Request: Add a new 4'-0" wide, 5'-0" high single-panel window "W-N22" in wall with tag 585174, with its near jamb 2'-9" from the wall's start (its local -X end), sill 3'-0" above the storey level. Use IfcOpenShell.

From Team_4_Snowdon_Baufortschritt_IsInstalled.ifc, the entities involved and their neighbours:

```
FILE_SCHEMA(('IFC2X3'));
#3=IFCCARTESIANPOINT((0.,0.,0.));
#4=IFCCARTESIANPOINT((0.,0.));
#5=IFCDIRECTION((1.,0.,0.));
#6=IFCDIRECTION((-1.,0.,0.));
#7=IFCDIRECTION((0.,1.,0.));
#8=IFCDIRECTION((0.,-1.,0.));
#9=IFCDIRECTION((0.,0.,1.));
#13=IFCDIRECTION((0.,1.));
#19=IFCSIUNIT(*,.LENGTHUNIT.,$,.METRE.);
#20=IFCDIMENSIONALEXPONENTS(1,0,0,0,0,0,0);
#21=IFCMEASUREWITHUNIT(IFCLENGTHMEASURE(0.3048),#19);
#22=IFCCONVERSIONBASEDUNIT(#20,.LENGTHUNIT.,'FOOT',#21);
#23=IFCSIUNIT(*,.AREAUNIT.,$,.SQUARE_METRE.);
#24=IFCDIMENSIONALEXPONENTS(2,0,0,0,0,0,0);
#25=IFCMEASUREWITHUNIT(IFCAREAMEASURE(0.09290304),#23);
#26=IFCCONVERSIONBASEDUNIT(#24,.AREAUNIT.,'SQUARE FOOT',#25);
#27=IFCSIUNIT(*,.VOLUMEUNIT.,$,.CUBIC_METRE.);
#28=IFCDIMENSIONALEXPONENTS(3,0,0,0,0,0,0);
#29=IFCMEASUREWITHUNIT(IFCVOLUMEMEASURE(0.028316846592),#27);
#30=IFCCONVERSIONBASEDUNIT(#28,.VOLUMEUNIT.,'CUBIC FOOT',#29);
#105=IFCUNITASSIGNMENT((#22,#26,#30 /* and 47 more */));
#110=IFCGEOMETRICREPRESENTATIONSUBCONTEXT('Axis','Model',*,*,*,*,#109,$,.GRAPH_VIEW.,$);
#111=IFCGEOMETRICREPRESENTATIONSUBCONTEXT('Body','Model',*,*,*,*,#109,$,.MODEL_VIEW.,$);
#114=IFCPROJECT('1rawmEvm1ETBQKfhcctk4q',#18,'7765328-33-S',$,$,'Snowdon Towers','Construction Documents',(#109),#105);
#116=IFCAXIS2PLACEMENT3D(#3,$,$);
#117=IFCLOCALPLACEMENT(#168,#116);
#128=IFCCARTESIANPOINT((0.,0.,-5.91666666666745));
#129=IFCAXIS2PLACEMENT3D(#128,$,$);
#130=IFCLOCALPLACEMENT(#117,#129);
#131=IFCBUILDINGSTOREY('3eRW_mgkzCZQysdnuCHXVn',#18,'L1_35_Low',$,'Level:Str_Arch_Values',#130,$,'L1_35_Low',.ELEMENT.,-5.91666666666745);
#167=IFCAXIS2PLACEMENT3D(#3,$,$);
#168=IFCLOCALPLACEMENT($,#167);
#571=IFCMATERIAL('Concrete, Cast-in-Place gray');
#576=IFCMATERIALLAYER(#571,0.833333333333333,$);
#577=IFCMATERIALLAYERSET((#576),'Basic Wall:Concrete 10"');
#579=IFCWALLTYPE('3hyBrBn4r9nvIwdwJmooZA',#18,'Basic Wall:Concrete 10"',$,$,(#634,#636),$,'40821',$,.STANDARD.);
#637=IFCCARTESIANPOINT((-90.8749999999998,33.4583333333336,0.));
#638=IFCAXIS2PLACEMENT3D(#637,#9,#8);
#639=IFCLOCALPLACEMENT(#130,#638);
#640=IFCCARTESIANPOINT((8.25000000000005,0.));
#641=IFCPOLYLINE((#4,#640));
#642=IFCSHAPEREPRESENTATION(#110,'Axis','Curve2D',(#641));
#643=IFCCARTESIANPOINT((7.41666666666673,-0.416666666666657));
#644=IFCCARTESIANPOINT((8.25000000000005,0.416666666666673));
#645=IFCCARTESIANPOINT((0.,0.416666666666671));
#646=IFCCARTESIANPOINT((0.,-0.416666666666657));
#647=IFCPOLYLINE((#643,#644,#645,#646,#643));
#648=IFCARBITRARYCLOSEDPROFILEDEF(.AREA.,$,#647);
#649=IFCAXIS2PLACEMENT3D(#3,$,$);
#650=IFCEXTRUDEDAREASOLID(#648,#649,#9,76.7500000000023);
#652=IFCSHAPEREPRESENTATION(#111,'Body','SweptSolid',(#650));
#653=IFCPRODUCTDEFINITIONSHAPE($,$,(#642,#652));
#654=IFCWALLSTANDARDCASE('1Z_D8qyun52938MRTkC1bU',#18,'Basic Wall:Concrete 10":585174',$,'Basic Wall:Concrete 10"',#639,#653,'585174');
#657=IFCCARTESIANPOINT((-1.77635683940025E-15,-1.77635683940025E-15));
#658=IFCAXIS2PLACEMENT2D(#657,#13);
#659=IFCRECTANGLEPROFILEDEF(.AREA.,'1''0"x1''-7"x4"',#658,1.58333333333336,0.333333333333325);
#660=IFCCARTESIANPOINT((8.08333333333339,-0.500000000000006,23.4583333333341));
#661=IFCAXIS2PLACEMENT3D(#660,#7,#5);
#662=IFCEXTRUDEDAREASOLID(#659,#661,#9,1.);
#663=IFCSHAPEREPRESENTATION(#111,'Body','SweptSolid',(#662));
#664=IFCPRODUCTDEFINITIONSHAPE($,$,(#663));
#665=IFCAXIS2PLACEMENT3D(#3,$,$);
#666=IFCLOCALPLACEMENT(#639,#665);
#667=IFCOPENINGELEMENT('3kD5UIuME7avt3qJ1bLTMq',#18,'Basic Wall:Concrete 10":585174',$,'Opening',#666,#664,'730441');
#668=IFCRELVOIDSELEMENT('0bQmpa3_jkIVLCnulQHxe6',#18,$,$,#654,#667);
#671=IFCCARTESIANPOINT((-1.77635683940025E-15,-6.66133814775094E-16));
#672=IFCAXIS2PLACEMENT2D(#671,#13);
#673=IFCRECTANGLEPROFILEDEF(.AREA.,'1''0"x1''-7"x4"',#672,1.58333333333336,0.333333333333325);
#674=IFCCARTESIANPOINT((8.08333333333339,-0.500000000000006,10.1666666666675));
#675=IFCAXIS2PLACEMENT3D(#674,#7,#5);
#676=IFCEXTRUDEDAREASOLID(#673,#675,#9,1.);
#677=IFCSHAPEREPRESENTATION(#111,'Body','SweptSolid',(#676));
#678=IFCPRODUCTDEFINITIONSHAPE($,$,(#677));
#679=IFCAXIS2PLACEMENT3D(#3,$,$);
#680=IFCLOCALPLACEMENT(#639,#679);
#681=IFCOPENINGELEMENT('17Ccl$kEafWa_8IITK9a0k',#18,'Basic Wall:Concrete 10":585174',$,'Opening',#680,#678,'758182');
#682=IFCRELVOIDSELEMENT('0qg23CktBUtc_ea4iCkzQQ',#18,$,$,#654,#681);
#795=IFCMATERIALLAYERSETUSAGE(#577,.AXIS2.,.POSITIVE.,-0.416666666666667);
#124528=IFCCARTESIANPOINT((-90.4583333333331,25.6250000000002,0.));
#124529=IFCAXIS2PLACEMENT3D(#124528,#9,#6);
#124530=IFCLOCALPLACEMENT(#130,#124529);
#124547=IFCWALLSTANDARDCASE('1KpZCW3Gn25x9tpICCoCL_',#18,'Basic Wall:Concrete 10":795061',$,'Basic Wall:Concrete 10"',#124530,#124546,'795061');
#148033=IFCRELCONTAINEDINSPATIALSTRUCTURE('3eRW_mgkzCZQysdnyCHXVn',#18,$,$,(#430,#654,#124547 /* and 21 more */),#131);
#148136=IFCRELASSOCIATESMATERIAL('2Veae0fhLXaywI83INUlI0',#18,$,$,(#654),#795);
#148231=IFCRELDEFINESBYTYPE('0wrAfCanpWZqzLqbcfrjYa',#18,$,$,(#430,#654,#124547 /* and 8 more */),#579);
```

```python
import numpy as np
import ifcopenshell
import ifcopenshell.api.feature
import ifcopenshell.api.geometry
import ifcopenshell.api.root
import ifcopenshell.api.spatial
import ifcopenshell.api.type
import ifcopenshell.geom
import ifcopenshell.util.element
import ifcopenshell.util.placement
import ifcopenshell.util.representation
import ifcopenshell.util.shape
import ifcopenshell.util.unit

model = ifcopenshell.open("Team_4_Snowdon_Baufortschritt_IsInstalled.ifc")
unit_scale = ifcopenshell.util.unit.calculate_unit_scale(model)
settings = ifcopenshell.geom.settings()


def volume(element):
    """Net volume in cubic metres, openings subtracted."""
    shape = ifcopenshell.geom.create_shape(settings, element)
    return ifcopenshell.util.shape.get_volume(shape.geometry)


wall = model.by_guid("1Z_D8qyun52938MRTkC1bU")
storey = ifcopenshell.util.element.get_container(wall, ifc_class="IfcBuildingStorey")
context = ifcopenshell.util.representation.get_context(model, "Model", "Body", "MODEL_VIEW")
before = volume(wall)

width, height, from_end, sill = 1.2192, 1.524, 0.8382, 0.9144  # metres

# The wall runs along its own X axis, and the end named is its -X end.
wall_shape = ifcopenshell.geom.create_shape(settings, wall)
x, y, z = ifcopenshell.util.shape.get_vertices(wall_shape.geometry).T
start = x.min() + from_end
face, thickness = float(y.min()), float(y.max() - y.min())
wall_matrix = ifcopenshell.util.placement.get_local_placement(wall.ObjectPlacement)
level = ifcopenshell.util.placement.get_local_placement(storey.ObjectPlacement)[2, 3]


def in_wall(x, y):
    """Placement at x, y metres in the wall's axes, at sill height."""
    matrix = wall_matrix.copy()
    matrix[:, 3] = wall_matrix @ np.array([x / unit_scale, y / unit_scale, 0.0, 1.0])
    matrix[2, 3] = level + sill / unit_scale
    return matrix


# Opening: a box that overshoots both wall faces by 50 mm.
opening = ifcopenshell.api.root.create_entity(model, ifc_class="IfcOpeningElement")
box = ifcopenshell.api.geometry.add_wall_representation(
    model, context=context, length=width, height=height, thickness=thickness + 0.1
)
ifcopenshell.api.geometry.assign_representation(model, product=opening, representation=box)
ifcopenshell.api.geometry.edit_object_placement(model, product=opening, matrix=in_wall(start, face - 0.05), is_si=False)
ifcopenshell.api.feature.add_feature(model, feature=opening, element=wall)

window = ifcopenshell.api.root.create_entity(model, ifc_class="IfcWindow", name="W-N22")
window.OverallWidth, window.OverallHeight = width / unit_scale, height / unit_scale
body = ifcopenshell.api.geometry.add_window_representation(
    model,
    context=context,
    overall_width=window.OverallWidth,
    overall_height=window.OverallHeight,
    partition_type="SINGLE_PANEL",
)
ifcopenshell.api.geometry.assign_representation(model, product=window, representation=body)
ifcopenshell.api.spatial.assign_container(model, products=[window], relating_structure=storey)
fills = ifcopenshell.api.feature.add_filling(model, opening=opening, element=window)
fills.OwnerHistory = window.OwnerHistory  # required in IFC2X3

# IFC2X3 keeps the operation on the window style.
style = ifcopenshell.api.root.create_entity(model, ifc_class="IfcWindowStyle", name="W-N22")
style.OperationType, style.ConstructionType = "SINGLE_PANEL", "NOTDEFINED"
style.ParameterTakesPrecedence = style.Sizeable = False
ifcopenshell.api.type.assign_type(model, related_objects=[window], relating_type=style)

# Centre the window in the wall's thickness.
ifcopenshell.api.geometry.edit_object_placement(model, product=window, matrix=in_wall(start, face), is_si=False)
window_shape = ifcopenshell.geom.create_shape(settings, window)
depth = ifcopenshell.util.shape.get_vertices(window_shape.geometry)[:, 1]
offset = face + thickness / 2 - (depth.min() + depth.max()) / 2
ifcopenshell.api.geometry.edit_object_placement(model, product=window, matrix=in_wall(start, offset), is_si=False)

after = volume(wall)

print(f"wall volume {before:.3f} -> {after:.3f} m3")

model.write("Team_4_Snowdon_Baufortschritt_IsInstalled_rev.ifc")
```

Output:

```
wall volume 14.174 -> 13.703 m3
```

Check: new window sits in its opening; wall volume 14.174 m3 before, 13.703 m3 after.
